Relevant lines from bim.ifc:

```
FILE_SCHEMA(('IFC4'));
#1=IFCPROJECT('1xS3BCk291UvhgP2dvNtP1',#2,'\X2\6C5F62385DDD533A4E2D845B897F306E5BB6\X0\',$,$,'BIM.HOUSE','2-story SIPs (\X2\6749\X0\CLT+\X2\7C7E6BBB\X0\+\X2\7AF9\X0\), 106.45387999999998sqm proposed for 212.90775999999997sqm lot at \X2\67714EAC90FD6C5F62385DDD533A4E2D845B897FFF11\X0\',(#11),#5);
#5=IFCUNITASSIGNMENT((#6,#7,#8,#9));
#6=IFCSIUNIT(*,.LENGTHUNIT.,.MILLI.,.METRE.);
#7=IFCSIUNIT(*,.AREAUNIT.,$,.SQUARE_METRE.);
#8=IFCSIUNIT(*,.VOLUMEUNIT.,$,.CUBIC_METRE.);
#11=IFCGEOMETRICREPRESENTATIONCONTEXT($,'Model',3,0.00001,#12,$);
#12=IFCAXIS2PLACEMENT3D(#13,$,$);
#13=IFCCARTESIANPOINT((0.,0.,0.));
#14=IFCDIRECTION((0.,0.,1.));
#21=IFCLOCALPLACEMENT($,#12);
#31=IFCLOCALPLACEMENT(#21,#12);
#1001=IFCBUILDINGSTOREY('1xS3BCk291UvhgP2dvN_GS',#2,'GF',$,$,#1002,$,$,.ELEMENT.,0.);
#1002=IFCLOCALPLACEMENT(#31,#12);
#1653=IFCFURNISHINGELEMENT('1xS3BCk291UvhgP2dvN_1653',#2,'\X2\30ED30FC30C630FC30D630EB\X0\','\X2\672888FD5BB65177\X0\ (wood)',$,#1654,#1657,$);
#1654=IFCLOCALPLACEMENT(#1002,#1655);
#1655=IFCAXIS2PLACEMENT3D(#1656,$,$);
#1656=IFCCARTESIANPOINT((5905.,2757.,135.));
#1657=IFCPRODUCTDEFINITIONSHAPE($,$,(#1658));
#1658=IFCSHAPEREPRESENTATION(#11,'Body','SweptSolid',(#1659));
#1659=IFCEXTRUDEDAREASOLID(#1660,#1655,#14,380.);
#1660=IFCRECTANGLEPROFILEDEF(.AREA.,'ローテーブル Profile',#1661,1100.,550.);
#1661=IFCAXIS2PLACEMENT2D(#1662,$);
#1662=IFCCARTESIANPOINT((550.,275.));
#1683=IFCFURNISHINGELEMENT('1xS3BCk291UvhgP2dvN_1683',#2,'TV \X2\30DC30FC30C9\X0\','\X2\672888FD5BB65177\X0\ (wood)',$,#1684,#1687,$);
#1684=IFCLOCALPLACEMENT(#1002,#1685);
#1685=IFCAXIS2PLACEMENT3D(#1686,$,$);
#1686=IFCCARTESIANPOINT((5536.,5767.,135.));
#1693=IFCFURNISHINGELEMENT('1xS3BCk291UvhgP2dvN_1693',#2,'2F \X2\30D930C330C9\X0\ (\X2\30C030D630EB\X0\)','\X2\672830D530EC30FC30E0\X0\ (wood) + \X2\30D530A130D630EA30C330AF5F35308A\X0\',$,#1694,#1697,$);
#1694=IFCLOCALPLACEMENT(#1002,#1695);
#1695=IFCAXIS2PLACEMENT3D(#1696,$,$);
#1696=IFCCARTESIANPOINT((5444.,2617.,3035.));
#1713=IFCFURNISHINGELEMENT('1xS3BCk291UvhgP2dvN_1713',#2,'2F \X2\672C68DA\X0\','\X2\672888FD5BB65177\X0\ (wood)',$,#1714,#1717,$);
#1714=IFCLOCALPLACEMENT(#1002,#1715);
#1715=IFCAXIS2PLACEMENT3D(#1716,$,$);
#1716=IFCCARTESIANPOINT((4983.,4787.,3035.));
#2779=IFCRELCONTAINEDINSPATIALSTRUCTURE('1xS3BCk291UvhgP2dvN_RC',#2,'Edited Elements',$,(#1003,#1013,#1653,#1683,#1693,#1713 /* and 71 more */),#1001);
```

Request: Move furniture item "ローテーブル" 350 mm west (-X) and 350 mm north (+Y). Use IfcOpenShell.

```python
import ifcopenshell
import ifcopenshell.api.geometry
import ifcopenshell.util.placement
import ifcopenshell.util.unit

model = ifcopenshell.open("bim.ifc")
unit_scale = ifcopenshell.util.unit.calculate_unit_scale(model)

item = model.by_id(1653)
matrix = ifcopenshell.util.placement.get_local_placement(item.ObjectPlacement)
matrix[0, 3] -= 0.35 / unit_scale
matrix[1, 3] += 0.35 / unit_scale
ifcopenshell.api.geometry.edit_object_placement(model, product=item, matrix=matrix, is_si=False)

print(ifcopenshell.util.placement.get_local_placement(item.ObjectPlacement).round(3) + 0.0)

model.write("bim_updated.ifc")
```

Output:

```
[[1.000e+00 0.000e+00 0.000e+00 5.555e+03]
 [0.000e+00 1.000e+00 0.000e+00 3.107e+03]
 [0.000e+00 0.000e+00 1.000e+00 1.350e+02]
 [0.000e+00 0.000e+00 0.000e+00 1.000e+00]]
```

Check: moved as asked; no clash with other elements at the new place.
